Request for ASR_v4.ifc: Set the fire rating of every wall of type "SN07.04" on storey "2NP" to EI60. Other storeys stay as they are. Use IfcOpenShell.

First a look at what the model holds.

```python
import ifcopenshell
import ifcopenshell.util.element

model = ifcopenshell.open("ASR_v4.ifc")
print(model.schema)
storey = next(s for s in model.by_type("IfcBuildingStorey") if s.Name == "2NP")
walls = [e for e in ifcopenshell.util.element.get_decomposition(storey) if e.is_a("IfcWall")]
seen = {}
for e in walls:
    element_type = ifcopenshell.util.element.get_type(e)
    key = (element_type.Name if element_type != e and element_type else None, ifcopenshell.util.element.get_pset(e, "Pset_WallCommon", "FireRating"))
    seen[key] = seen.get(key, 0) + 1
for (name, value), count in sorted(seen.items(), key=str):
    print(count, "x", name, "|", value)
```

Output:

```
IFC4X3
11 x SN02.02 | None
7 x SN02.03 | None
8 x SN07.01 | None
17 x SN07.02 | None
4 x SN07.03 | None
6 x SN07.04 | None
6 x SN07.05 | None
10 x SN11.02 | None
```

```python
import ifcopenshell
import ifcopenshell.api.pset
import ifcopenshell.util.element

model = ifcopenshell.open("ASR_v4.ifc")

storey = next(s for s in model.by_type("IfcBuildingStorey") if s.Name == "2NP")
walls = [e for e in ifcopenshell.util.element.get_decomposition(storey) if e.is_a("IfcWall")]

count = 0
for e in walls:
    element_type = ifcopenshell.util.element.get_type(e)
    if element_type in (None, e) or element_type.Name != "SN07.04":
        continue
    # add_pset returns the element's existing set when there is one.
    pset = ifcopenshell.api.pset.add_pset(model, product=e, name="Pset_WallCommon")
    ifcopenshell.api.pset.edit_pset(model, pset=pset, properties={"FireRating": "EI60"})
    count += 1

print(count, "walls updated")

model.write("ASR_v4_updated.ifc")
```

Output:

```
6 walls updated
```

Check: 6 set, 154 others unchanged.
